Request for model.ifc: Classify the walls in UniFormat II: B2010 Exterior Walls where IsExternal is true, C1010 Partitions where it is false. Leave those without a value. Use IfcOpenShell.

First a look at what the model holds.

```python
import ifcopenshell
import ifcopenshell.util.element

model = ifcopenshell.open("model.ifc")
print(model.schema)
print("classifications:", [c.Name for c in model.by_type("IfcClassification")])
values = [ifcopenshell.util.element.get_pset(e, "Pset_WallCommon", "IsExternal") for e in model.by_type("IfcWall")]
for value in (True, False, None):
    print("IsExternal", value, values.count(value))
```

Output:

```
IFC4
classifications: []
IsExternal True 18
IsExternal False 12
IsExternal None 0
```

```python
import ifcopenshell
import ifcopenshell.api.classification
import ifcopenshell.util.element

model = ifcopenshell.open("model.ifc")

system = ifcopenshell.api.classification.add_classification(model, classification="UniFormat II")

walls = model.by_type("IfcWall")
external = {e: ifcopenshell.util.element.get_pset(e, "Pset_WallCommon", "IsExternal") for e in walls}
for flag, code, name in ((True, "B2010", "Exterior Walls"), (False, "C1010", "Partitions")):
    products = [e for e in walls if external[e] is flag]
    ifcopenshell.api.classification.add_reference(
        model, products=products, classification=system, identification=code, name=name
    )
    print(code, len(products))

model.write("model_v2.ifc")
```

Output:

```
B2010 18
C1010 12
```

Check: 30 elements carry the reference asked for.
